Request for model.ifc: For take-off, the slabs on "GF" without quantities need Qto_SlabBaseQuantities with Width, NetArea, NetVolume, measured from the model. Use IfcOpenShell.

First a look at what the model holds.

```python
import ifcopenshell
import ifcopenshell.util.element
import ifcopenshell.util.unit

model = ifcopenshell.open("model.ifc")
print(model.schema)
for unit_type in ("LENGTHUNIT", "AREAUNIT", "VOLUMEUNIT"):
    print(unit_type, ifcopenshell.util.unit.calculate_unit_scale(model, unit_type))
storey = next(s for s in model.by_type("IfcBuildingStorey") if s.Name == "GF")
slabs = [e for e in ifcopenshell.util.element.get_decomposition(storey) if e.is_a("IfcSlab")]
for e in sorted(slabs, key=lambda e: e.id()):
    print(e.id(), e.is_a(), e.Name, list(ifcopenshell.util.element.get_psets(e, qtos_only=True)), sep=" | ")
```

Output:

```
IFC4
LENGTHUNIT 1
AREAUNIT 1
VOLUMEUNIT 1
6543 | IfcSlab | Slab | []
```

```python
import ifcopenshell
import ifcopenshell.api.pset
import ifcopenshell.geom
import ifcopenshell.util.element
import ifcopenshell.util.shape
import ifcopenshell.util.unit

model = ifcopenshell.open("model.ifc")
unit_scale = ifcopenshell.util.unit.calculate_unit_scale(model)
area_scale = ifcopenshell.util.unit.calculate_unit_scale(model, "AREAUNIT")
volume_scale = ifcopenshell.util.unit.calculate_unit_scale(model, "VOLUMEUNIT")
settings = ifcopenshell.geom.settings()

storey = next(s for s in model.by_type("IfcBuildingStorey") if s.Name == "GF")
slabs = [e for e in ifcopenshell.util.element.get_decomposition(storey) if e.is_a("IfcSlab")]

for e in sorted(slabs, key=lambda e: e.id()):
    if ifcopenshell.util.element.get_psets(e, qtos_only=True, should_inherit=False):
        continue
    # Geometry comes back in metres, in the element's own axes.
    shape = ifcopenshell.geom.create_shape(settings, e)
    values = {
        "Width": ifcopenshell.util.shape.get_z(shape.geometry) / unit_scale,
        "NetArea": ifcopenshell.util.shape.get_footprint_area(shape.geometry) / area_scale,
        "NetVolume": ifcopenshell.util.shape.get_volume(shape.geometry) / volume_scale,
    }
    qto = ifcopenshell.api.pset.add_qto(model, product=e, name="Qto_SlabBaseQuantities")
    ifcopenshell.api.pset.edit_qto(model, qto=qto, properties=values)
    print(e.id(), {k: round(v, 3) for k, v in values.items()})

model.write("model_updated.ifc")
```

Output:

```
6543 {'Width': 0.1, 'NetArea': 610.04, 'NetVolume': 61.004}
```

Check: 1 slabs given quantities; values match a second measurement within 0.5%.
